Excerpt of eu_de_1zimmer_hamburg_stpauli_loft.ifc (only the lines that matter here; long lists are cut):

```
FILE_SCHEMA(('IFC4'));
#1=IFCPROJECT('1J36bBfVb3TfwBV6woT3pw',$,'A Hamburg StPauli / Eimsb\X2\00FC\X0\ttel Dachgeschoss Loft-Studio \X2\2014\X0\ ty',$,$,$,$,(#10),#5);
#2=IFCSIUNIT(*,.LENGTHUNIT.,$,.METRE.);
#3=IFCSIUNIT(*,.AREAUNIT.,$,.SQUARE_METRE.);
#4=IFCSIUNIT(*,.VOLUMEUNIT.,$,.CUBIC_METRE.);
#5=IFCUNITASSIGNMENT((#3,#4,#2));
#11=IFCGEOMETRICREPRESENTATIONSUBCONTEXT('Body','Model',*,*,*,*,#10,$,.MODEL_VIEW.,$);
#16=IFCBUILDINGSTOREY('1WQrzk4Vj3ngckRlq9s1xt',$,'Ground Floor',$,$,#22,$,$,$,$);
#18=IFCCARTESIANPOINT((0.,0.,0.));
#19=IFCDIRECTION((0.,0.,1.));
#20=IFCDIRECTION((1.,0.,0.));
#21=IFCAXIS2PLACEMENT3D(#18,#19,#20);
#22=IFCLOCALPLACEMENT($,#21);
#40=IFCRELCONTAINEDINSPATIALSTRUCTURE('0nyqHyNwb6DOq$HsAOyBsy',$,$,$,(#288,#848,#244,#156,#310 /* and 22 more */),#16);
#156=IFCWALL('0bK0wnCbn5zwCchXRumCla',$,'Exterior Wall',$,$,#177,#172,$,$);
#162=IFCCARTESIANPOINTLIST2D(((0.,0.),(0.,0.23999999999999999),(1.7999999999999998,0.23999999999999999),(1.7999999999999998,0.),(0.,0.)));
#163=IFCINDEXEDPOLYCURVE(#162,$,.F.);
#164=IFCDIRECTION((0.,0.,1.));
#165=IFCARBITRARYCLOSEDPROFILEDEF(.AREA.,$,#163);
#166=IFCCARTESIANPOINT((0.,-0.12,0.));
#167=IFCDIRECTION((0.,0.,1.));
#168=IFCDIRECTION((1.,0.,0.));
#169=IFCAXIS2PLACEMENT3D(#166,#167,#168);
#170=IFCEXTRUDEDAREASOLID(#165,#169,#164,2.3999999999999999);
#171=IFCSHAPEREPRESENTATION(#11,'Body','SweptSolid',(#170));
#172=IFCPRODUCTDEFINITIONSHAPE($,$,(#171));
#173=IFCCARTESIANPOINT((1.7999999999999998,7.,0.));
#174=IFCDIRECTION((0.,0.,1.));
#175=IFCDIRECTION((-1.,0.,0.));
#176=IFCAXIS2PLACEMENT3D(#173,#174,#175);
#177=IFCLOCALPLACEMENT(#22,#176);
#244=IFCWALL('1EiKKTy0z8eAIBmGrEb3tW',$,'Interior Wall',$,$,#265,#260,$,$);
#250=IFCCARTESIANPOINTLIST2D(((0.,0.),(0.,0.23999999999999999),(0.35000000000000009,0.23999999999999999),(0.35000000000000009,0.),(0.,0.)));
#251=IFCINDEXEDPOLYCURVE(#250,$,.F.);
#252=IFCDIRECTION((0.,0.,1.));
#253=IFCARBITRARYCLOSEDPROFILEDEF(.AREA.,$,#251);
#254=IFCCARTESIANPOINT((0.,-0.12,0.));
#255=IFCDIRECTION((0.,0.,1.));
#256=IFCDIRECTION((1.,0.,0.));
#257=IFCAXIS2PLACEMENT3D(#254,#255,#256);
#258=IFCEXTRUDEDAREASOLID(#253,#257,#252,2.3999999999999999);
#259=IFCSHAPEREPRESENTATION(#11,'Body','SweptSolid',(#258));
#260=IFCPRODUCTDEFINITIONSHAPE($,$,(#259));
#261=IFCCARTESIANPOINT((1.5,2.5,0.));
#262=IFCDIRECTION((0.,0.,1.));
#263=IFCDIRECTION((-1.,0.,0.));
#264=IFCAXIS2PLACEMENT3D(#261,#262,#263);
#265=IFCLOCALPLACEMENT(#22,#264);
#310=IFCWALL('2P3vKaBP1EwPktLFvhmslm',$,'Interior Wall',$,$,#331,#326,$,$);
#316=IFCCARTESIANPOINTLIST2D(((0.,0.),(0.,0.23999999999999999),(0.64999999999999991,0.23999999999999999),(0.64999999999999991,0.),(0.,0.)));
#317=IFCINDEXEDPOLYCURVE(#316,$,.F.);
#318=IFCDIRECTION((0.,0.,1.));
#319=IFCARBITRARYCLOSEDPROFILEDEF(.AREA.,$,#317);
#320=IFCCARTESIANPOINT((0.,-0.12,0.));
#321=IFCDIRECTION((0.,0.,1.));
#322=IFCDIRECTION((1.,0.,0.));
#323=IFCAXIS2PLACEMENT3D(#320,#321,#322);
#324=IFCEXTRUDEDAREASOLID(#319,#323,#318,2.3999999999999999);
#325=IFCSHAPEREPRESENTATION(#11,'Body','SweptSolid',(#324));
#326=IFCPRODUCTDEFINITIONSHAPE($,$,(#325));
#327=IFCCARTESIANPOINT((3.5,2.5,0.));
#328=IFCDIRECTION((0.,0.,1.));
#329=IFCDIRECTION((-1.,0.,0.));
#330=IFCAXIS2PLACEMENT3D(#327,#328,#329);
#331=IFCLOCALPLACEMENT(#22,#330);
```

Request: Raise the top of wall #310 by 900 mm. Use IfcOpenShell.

```python
import ifcopenshell
import ifcopenshell.geom
import ifcopenshell.util.representation
import ifcopenshell.util.shape
import ifcopenshell.util.unit

model = ifcopenshell.open("eu_de_1zimmer_hamburg_stpauli_loft.ifc")
unit_scale = ifcopenshell.util.unit.calculate_unit_scale(model)
settings = ifcopenshell.geom.settings()


def volume(element):
    """Net volume in cubic metres, openings subtracted."""
    shape = ifcopenshell.geom.create_shape(settings, element)
    return ifcopenshell.util.shape.get_volume(shape.geometry)


wall = model.by_id(310)
before = volume(wall)

body = ifcopenshell.util.representation.get_representation(wall, "Model", "Body")
solid = body.Items[0]
old_height = solid.Depth
solid.Depth += 0.9 / unit_scale
after = volume(wall)

print(f"height {old_height:g} -> {solid.Depth:g}, volume {before:.3f} -> {after:.3f} m3")

model.write("eu_de_1zimmer_hamburg_stpauli_loft_v2.ifc")
```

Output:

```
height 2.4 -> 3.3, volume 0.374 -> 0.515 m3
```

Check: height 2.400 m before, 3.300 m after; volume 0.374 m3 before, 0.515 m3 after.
